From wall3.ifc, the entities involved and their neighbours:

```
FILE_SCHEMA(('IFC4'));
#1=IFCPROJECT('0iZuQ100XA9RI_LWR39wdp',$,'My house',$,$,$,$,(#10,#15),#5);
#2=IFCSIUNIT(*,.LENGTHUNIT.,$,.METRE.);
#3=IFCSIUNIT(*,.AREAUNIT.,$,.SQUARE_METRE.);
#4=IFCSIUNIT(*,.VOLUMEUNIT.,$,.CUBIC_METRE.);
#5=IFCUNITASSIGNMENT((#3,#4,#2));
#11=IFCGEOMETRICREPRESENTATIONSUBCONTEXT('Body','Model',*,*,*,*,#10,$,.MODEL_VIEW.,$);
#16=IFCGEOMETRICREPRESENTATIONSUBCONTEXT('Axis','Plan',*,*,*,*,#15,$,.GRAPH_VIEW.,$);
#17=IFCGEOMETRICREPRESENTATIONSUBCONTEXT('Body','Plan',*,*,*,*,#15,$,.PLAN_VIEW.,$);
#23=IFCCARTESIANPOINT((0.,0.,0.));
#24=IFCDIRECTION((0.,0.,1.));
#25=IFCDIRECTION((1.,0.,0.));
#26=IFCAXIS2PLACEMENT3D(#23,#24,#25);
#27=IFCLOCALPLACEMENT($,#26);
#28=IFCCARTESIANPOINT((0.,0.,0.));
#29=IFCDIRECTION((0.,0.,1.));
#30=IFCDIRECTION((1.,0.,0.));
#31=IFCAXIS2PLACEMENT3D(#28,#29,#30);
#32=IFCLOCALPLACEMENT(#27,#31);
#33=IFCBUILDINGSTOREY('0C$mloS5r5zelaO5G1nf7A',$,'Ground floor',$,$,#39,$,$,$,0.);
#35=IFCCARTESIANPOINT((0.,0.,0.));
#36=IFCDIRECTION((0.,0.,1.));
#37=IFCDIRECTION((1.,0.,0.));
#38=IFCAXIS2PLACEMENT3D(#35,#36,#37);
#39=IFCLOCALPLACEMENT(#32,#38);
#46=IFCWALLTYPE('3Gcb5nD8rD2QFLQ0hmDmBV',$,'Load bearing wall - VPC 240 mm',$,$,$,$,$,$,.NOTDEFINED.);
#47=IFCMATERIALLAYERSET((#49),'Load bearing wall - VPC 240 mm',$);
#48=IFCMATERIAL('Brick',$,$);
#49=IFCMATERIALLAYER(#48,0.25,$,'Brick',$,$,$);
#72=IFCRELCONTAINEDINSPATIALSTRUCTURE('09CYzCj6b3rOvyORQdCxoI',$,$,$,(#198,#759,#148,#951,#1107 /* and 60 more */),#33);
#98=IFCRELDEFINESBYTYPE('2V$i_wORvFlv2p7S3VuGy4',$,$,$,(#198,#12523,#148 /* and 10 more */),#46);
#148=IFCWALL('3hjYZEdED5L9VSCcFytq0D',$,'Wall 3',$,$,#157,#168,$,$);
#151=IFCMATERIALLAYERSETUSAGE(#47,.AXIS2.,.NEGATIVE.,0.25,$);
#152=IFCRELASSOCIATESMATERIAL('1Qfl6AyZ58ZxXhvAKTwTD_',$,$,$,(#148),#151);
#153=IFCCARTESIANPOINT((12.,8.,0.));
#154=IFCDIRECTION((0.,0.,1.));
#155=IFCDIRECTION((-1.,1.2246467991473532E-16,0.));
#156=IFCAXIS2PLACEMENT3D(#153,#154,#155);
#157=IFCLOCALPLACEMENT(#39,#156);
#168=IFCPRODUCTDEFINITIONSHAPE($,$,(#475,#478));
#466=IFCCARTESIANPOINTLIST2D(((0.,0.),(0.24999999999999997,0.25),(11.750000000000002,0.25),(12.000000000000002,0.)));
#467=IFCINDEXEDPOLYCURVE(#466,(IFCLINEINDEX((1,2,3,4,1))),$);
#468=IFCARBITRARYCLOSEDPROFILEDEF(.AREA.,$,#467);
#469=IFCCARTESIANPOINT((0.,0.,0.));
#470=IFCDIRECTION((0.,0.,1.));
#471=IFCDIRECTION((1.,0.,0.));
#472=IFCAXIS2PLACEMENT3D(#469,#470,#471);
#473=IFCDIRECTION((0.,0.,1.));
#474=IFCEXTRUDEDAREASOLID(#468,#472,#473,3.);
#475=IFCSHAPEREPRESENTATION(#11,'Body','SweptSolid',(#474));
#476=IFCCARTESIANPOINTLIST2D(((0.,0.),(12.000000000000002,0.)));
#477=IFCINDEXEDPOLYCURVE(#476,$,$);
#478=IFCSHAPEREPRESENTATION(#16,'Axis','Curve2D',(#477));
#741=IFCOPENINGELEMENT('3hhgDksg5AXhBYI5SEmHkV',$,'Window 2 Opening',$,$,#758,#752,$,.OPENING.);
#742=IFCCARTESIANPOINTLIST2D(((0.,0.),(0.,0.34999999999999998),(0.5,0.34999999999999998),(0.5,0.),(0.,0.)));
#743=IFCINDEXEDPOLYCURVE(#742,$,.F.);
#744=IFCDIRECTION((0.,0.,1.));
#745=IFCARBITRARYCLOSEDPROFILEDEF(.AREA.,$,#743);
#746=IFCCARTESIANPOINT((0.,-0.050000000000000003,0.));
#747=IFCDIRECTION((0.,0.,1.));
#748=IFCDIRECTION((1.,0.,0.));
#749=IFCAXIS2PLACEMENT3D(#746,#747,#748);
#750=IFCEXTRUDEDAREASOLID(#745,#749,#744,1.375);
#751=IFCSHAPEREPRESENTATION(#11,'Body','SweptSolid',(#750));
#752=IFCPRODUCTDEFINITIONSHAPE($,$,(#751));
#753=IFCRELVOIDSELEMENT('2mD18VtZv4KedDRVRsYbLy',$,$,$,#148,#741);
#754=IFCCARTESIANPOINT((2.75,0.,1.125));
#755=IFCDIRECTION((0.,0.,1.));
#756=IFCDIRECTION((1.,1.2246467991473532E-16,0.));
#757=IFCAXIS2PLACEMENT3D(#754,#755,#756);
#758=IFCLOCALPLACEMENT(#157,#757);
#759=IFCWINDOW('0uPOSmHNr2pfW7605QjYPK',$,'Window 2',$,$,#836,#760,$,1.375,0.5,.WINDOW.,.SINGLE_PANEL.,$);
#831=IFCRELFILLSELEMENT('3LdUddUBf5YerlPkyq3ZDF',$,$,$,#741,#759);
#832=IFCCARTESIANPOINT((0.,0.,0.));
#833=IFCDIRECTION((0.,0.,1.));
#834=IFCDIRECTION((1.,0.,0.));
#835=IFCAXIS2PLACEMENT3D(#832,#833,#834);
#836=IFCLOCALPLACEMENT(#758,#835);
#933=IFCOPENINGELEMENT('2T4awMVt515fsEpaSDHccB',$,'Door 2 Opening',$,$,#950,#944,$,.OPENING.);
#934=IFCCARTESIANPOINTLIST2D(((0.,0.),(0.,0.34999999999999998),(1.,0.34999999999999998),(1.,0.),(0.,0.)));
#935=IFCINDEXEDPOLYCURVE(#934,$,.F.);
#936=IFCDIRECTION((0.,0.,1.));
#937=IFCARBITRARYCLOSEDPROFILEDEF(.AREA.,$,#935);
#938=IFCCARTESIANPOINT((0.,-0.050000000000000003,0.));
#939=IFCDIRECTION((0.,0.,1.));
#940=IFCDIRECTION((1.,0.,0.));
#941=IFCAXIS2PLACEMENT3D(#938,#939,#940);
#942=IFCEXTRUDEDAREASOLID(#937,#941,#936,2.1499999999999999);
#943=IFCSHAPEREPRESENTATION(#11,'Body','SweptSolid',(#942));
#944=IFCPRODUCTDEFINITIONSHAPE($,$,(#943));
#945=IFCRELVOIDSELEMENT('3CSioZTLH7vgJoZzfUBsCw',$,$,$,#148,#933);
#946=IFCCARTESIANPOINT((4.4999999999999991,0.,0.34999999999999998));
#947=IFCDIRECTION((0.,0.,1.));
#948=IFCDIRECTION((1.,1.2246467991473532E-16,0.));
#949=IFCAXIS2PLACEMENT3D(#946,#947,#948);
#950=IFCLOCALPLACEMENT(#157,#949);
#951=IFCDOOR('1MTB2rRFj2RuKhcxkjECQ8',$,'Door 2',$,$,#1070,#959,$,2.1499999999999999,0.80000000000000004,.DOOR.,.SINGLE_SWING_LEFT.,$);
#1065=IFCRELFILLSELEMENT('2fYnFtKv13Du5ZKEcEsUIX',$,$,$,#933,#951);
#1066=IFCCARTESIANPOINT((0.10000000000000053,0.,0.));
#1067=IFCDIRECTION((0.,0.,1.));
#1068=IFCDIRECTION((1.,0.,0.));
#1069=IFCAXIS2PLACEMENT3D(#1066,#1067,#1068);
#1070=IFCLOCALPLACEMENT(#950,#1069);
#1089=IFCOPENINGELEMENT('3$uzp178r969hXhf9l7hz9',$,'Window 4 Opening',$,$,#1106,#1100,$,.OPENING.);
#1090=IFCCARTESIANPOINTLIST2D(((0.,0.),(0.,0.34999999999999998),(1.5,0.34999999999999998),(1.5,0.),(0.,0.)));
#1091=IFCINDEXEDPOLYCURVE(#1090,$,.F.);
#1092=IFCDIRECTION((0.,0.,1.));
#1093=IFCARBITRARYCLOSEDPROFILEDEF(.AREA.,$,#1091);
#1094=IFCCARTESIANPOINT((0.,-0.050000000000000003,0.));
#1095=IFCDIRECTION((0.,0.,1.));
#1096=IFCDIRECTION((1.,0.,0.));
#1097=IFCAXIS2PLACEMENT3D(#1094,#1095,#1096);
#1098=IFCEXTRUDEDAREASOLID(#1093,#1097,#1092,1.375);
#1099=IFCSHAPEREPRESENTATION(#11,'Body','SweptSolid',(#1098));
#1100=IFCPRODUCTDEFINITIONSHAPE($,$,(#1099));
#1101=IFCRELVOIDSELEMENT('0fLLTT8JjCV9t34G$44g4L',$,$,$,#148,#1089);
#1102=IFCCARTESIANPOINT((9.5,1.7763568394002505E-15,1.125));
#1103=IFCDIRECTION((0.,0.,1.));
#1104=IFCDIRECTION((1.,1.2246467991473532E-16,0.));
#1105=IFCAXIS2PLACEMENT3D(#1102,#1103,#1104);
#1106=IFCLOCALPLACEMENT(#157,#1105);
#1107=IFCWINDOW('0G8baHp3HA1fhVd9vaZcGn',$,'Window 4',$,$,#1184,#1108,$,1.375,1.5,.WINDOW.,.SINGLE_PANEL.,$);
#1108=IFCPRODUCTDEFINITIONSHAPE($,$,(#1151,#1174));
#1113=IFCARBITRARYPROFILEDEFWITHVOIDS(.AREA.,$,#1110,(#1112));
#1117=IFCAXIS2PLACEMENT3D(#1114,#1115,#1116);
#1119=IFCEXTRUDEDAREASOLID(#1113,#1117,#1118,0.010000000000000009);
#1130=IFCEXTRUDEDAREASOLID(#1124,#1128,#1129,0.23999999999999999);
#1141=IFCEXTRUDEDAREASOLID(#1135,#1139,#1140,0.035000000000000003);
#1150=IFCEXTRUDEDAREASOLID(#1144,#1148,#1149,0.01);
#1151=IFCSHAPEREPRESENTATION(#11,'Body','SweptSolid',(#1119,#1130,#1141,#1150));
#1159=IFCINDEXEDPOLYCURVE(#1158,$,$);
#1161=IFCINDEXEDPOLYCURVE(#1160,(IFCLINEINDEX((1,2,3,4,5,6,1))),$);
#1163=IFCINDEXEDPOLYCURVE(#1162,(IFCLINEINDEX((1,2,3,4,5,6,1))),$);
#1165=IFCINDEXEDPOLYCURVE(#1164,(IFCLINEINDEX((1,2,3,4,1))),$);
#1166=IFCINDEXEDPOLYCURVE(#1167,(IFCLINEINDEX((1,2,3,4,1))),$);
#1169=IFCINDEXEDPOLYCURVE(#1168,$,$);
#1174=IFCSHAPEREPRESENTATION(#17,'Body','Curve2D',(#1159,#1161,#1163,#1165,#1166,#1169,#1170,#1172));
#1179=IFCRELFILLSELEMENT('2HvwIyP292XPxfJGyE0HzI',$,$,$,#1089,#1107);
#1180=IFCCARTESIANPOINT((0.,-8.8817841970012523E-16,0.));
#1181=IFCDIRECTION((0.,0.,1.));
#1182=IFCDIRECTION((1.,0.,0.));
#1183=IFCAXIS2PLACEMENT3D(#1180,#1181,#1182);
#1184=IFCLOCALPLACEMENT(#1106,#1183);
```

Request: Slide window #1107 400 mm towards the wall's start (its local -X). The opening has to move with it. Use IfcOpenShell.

```python
import ifcopenshell
import ifcopenshell.api.geometry
import ifcopenshell.util.placement
import ifcopenshell.util.unit

model = ifcopenshell.open("wall3.ifc")
unit_scale = ifcopenshell.util.unit.calculate_unit_scale(model)

window = model.by_guid("0G8baHp3HA1fhVd9vaZcGn")
opening = window.FillsVoids[0].RelatingOpeningElement
wall = opening.VoidsElements[0].RelatingBuildingElement

wall_matrix = ifcopenshell.util.placement.get_local_placement(wall.ObjectPlacement)
shift = wall_matrix[:3, 0] * -0.4 / unit_scale
before = ifcopenshell.util.placement.get_local_placement(window.ObjectPlacement)[:3, 3].copy()

# The window is placed relative to its opening, so it follows when the opening moves.
matrix = ifcopenshell.util.placement.get_local_placement(opening.ObjectPlacement)
matrix[:3, 3] += shift
ifcopenshell.api.geometry.edit_object_placement(
    model, product=opening, matrix=matrix, is_si=False, should_transform_children=True
)

after = ifcopenshell.util.placement.get_local_placement(window.ObjectPlacement)[:3, 3]
print("window moved by", (after - before).round(3) + 0.0)

model.write("wall3_updated.ifc")
```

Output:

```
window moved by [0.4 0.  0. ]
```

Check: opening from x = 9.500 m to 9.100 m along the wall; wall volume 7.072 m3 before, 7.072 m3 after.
